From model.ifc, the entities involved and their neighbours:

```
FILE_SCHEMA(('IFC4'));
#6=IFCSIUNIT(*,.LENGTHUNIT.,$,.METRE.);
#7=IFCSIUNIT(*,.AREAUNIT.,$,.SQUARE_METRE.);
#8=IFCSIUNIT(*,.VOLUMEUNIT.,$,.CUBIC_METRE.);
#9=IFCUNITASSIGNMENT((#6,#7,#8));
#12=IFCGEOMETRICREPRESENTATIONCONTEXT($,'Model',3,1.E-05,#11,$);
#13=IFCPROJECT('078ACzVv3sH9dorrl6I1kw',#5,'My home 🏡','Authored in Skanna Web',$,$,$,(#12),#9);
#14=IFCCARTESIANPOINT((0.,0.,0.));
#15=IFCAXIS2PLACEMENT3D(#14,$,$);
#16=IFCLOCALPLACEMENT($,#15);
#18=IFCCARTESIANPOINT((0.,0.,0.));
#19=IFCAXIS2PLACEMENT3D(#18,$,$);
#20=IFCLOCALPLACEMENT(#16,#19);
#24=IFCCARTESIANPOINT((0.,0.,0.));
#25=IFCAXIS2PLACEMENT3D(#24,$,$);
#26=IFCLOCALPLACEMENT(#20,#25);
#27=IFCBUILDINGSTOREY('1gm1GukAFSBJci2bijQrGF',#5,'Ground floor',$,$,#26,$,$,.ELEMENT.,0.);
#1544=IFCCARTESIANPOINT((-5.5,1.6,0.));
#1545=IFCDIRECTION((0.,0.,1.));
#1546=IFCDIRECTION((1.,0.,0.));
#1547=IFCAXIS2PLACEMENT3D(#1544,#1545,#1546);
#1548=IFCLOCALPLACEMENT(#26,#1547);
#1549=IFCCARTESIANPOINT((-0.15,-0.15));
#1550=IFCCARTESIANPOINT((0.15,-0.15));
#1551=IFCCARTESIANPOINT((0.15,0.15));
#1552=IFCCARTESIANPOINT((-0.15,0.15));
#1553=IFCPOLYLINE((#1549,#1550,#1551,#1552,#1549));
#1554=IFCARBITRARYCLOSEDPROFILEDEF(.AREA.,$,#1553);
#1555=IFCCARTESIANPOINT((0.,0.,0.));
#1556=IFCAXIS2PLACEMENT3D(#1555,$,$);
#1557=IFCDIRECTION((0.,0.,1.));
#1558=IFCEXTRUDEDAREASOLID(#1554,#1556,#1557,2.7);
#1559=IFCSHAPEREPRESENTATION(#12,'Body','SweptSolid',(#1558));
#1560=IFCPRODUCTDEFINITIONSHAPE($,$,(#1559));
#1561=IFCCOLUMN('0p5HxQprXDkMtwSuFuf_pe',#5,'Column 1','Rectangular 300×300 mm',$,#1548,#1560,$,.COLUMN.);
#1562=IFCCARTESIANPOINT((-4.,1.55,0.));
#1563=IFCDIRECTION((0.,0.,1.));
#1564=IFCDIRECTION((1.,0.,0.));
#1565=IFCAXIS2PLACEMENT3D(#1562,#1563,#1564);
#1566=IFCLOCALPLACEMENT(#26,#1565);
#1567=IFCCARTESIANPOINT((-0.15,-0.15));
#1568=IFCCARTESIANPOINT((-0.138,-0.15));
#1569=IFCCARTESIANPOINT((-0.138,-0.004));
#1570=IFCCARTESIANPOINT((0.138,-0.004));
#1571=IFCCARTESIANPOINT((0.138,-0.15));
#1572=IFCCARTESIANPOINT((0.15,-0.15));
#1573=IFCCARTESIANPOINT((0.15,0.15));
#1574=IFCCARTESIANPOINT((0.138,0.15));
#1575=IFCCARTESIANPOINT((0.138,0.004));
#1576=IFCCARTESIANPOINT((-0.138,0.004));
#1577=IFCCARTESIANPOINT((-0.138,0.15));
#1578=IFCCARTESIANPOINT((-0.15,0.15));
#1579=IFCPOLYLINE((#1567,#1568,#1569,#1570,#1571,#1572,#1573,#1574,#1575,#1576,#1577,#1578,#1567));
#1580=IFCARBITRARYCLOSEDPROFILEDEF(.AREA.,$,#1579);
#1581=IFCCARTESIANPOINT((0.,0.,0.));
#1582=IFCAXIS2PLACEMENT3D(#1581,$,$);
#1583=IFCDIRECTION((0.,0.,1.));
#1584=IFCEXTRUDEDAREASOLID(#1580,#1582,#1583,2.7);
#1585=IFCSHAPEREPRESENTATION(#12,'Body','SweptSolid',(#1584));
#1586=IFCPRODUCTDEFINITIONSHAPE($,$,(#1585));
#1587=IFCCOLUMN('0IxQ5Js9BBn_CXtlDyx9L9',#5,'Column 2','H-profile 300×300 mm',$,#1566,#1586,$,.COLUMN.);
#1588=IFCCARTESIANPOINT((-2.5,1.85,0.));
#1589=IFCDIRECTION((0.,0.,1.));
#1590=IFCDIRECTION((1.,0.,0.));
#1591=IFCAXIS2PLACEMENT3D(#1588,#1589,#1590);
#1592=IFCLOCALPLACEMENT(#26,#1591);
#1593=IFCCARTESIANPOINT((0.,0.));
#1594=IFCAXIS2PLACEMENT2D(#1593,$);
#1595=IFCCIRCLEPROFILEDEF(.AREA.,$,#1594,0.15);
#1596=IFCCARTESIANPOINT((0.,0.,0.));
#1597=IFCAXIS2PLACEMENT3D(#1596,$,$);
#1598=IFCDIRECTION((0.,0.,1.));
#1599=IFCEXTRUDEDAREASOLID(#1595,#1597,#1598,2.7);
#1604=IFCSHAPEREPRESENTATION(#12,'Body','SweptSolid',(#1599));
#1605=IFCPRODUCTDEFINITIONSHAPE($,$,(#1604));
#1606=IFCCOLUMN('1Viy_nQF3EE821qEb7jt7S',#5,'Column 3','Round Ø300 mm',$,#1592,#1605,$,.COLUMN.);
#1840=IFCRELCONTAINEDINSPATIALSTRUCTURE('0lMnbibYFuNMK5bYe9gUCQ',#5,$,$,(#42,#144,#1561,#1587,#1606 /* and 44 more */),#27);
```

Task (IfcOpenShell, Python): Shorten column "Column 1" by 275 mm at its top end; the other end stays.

```python
import ifcopenshell

model = ifcopenshell.open("model.ifc")

member = model.by_id(1561)
change = -0.275

# The extrusion runs towards the end named, so only its depth changes.
body = next(r for r in member.Representation.Representations if r.RepresentationIdentifier == "Body")
solid = body.Items[0]
old_length = solid.Depth
solid.Depth += change

print(f"length {old_length:g} -> {solid.Depth:g}")

model.write("model_edited.ifc")
```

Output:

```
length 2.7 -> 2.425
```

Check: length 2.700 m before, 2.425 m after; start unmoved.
